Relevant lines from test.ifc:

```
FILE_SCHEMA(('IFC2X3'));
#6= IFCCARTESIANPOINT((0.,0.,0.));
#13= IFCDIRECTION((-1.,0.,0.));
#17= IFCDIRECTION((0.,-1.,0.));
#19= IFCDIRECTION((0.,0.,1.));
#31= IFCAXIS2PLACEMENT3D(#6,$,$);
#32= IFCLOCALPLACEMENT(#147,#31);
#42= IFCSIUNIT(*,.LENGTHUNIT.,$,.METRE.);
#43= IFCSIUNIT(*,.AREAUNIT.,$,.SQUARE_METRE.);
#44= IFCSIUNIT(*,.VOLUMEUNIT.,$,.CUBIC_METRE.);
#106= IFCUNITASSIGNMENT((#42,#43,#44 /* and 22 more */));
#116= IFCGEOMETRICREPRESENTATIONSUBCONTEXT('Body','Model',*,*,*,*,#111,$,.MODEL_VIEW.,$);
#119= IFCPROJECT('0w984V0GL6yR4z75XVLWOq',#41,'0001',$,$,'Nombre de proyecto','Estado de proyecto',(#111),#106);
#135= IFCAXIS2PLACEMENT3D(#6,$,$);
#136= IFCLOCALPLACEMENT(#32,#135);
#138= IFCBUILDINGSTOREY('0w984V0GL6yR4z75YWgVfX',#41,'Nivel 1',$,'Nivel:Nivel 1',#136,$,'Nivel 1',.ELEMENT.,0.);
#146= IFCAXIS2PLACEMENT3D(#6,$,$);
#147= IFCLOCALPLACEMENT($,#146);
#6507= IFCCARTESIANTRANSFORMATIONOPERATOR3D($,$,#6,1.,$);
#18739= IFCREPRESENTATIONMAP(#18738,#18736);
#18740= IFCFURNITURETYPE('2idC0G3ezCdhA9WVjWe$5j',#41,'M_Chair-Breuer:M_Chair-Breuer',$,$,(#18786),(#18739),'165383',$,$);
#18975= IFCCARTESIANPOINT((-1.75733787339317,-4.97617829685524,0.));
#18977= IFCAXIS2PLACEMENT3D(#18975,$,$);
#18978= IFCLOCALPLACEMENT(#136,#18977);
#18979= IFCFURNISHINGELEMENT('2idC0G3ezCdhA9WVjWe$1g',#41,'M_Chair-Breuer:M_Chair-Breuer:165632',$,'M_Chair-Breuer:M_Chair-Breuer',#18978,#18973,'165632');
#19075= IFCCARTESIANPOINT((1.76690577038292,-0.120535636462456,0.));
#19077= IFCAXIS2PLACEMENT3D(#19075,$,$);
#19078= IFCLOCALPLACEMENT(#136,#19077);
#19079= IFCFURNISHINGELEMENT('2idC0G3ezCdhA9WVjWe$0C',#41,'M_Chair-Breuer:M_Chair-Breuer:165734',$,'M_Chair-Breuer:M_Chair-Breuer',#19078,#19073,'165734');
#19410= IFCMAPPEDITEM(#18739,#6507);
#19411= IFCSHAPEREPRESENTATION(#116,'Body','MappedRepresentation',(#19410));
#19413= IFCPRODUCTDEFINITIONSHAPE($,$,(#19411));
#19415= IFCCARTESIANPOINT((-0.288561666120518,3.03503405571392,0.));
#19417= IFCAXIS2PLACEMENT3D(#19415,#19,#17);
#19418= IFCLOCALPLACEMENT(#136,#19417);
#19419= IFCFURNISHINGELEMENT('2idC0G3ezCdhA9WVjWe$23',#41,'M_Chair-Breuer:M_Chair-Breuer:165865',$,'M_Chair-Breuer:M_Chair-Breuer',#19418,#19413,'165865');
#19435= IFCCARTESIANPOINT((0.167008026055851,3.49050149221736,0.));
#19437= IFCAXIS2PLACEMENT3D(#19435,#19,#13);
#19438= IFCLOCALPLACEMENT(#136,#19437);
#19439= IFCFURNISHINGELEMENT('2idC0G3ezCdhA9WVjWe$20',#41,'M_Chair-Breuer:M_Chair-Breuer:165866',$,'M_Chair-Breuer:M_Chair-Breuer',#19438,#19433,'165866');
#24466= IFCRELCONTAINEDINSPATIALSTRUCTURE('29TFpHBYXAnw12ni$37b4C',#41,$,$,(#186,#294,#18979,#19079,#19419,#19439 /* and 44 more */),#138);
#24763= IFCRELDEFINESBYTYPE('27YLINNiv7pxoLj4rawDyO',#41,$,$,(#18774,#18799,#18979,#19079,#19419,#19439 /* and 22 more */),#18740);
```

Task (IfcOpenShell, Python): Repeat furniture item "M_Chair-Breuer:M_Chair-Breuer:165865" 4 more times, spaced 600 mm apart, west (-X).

```python
import numpy as np
import ifcopenshell
import ifcopenshell.api.geometry
import ifcopenshell.api.root
import ifcopenshell.util.element
import ifcopenshell.util.placement
import ifcopenshell.util.unit

model = ifcopenshell.open("test.ifc")
unit_scale = ifcopenshell.util.unit.calculate_unit_scale(model)


def reuse_history(source, copy):
    """copy_class also copies each property set's owner history, people and application; keep the originals."""
    for rel in copy.IsDefinedBy:
        if rel.is_a("IfcRelDefinesByProperties") and (history := rel.RelatingPropertyDefinition.OwnerHistory):
            rel.RelatingPropertyDefinition.OwnerHistory = source.OwnerHistory
            ifcopenshell.util.element.remove_deep2(model, history)


source = model.by_guid("2idC0G3ezCdhA9WVjWe$23")
base = ifcopenshell.util.placement.get_local_placement(source.ObjectPlacement)
step = np.array([-1.0, 0.0, 0.0]) * 0.6 / unit_scale

for i in range(1, 5):
    copy = ifcopenshell.api.root.copy_class(model, product=source)
    copy.Representation = ifcopenshell.util.element.copy_deep(
        model, source.Representation, exclude=["IfcGeometricRepresentationContext", "IfcRepresentationMap"]
    )
    copy.Name = "M_Chair-Breuer:M_Chair-Breuer"
    copy.Tag = None
    reuse_history(source, copy)
    matrix = base.copy()
    matrix[:3, 3] += i * step
    print("added at", matrix[:3, 3].round(3) + 0.0)
    ifcopenshell.api.geometry.edit_object_placement(model, product=copy, matrix=matrix, is_si=False)

model.write("test_rev.ifc")
```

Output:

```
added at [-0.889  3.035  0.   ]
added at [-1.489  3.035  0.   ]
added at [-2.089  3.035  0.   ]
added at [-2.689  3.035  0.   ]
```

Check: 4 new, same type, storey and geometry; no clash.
